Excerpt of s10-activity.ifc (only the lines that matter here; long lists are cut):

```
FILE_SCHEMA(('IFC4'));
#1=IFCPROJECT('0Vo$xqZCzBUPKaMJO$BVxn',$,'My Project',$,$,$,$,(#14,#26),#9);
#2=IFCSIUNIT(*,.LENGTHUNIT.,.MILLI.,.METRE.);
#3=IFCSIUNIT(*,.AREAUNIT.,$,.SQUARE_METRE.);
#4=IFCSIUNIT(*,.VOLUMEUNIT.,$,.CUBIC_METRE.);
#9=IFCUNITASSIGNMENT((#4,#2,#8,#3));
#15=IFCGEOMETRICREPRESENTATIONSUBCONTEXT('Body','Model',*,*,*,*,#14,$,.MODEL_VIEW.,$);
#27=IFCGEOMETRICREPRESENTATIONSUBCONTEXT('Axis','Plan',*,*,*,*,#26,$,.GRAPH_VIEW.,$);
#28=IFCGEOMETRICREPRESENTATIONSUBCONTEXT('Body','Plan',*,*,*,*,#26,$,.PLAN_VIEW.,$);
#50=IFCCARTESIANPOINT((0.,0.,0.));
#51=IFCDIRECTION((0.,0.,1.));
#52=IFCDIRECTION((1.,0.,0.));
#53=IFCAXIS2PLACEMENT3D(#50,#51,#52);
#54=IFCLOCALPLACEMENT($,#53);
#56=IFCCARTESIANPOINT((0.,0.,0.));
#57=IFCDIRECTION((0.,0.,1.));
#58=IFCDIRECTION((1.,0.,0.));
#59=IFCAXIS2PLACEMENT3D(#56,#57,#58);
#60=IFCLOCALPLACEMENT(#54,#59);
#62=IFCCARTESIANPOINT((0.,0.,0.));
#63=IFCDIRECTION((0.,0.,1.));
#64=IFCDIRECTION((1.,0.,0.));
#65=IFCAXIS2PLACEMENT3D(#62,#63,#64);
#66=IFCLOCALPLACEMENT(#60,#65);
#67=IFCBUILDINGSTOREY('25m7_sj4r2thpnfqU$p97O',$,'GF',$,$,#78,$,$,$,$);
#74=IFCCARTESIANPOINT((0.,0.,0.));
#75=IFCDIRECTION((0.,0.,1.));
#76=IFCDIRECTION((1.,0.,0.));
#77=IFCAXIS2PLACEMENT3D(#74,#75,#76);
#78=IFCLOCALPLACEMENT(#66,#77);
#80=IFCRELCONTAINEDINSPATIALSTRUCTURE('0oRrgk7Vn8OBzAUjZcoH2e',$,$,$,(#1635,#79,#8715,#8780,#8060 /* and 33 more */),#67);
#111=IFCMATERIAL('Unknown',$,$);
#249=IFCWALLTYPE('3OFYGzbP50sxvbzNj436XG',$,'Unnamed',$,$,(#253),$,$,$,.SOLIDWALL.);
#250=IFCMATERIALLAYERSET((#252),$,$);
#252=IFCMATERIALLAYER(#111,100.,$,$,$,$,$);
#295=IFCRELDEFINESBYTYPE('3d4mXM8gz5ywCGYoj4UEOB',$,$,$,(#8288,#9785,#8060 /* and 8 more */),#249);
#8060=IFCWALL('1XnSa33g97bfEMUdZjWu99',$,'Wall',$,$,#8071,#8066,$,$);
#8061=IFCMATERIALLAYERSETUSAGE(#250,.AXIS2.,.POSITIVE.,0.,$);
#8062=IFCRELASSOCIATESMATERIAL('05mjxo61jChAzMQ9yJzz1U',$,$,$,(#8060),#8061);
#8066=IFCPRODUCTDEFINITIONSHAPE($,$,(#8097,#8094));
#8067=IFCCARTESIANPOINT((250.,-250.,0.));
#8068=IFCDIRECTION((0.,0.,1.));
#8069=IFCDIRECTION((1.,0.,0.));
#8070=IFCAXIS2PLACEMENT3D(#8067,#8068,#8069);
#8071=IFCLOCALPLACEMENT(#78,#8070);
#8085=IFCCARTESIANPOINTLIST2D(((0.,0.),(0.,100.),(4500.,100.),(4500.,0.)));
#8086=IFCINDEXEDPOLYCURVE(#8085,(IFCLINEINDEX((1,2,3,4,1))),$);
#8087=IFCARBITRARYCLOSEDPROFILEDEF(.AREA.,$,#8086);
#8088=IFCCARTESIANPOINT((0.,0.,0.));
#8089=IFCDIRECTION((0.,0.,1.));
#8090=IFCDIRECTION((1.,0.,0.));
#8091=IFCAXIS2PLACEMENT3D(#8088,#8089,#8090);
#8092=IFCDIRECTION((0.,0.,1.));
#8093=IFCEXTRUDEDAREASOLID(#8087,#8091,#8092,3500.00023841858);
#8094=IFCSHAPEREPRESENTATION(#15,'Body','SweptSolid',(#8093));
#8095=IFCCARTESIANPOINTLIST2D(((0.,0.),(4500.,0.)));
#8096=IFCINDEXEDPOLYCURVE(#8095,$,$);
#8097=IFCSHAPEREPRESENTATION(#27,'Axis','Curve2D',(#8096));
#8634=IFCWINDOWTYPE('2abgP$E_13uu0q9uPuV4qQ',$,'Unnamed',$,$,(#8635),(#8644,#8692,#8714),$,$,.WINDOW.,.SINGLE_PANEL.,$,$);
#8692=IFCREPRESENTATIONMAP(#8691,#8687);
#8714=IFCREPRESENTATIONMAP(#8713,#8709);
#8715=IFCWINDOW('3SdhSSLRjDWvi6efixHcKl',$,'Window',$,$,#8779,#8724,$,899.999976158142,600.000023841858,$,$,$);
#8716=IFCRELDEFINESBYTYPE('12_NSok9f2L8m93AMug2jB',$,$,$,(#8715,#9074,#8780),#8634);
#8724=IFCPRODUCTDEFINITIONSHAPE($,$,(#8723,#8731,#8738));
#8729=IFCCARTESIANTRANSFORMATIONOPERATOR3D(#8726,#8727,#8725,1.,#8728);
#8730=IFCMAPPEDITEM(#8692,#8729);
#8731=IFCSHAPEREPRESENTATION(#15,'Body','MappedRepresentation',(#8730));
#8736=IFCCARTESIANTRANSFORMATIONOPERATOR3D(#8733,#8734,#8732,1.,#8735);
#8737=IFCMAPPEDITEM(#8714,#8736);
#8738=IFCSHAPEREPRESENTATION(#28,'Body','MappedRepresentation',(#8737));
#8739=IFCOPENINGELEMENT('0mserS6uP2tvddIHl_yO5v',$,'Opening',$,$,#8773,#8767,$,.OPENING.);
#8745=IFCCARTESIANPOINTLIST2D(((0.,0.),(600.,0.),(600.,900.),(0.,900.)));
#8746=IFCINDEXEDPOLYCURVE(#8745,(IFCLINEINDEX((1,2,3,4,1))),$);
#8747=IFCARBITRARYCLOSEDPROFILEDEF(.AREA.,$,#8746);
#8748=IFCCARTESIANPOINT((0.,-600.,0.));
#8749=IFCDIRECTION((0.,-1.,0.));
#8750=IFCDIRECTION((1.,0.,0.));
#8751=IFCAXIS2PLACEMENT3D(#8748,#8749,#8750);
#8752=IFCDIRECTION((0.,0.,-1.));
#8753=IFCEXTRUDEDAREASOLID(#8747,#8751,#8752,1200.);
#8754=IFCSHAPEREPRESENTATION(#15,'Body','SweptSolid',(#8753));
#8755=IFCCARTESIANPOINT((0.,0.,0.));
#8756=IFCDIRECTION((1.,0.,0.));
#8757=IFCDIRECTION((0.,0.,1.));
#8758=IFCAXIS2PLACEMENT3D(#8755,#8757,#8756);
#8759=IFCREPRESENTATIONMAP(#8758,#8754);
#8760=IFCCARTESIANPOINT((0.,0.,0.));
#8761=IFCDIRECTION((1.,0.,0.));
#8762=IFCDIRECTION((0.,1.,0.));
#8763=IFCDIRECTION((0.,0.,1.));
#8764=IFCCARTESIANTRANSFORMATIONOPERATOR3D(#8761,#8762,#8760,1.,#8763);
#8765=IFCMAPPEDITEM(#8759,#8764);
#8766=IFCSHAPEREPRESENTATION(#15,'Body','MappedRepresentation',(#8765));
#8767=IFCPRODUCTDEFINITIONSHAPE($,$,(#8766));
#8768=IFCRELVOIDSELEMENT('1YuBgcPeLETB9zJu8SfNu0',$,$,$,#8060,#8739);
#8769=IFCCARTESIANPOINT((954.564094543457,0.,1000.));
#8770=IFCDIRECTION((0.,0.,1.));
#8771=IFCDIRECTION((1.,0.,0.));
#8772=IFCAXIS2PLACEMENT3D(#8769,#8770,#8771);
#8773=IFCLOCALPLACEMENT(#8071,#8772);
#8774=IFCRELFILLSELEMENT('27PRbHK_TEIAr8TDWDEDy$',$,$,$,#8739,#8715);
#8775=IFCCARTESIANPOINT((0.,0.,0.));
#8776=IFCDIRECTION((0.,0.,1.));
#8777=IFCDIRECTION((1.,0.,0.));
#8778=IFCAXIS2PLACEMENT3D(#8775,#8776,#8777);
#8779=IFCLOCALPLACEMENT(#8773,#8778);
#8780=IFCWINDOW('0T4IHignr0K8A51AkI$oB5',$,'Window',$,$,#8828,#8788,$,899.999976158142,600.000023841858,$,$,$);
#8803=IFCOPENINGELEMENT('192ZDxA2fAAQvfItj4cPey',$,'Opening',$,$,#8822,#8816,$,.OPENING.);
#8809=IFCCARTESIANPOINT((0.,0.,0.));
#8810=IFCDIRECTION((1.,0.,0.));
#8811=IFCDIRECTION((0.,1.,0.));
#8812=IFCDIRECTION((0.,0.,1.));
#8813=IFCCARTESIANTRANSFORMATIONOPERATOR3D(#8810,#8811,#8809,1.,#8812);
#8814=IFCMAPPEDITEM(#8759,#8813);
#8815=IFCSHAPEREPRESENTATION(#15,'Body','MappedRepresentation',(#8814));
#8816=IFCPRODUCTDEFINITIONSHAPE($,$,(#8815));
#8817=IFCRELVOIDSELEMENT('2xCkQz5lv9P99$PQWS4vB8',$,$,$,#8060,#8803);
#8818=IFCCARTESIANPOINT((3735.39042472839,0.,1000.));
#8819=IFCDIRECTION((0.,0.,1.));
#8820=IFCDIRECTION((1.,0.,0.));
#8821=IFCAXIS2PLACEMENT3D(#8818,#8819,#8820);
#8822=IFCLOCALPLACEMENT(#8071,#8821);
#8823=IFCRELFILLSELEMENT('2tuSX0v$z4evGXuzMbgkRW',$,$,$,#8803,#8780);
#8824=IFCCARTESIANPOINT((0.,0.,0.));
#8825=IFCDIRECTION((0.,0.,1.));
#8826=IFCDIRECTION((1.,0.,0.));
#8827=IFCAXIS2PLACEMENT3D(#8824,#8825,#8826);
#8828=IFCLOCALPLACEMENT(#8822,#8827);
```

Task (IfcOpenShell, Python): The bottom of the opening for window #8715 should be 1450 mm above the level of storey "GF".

```python
import numpy as np
import ifcopenshell
import ifcopenshell.api.geometry
import ifcopenshell.geom
import ifcopenshell.util.element
import ifcopenshell.util.placement
import ifcopenshell.util.shape
import ifcopenshell.util.unit

model = ifcopenshell.open("s10-activity.ifc")
unit_scale = ifcopenshell.util.unit.calculate_unit_scale(model)

window = model.by_id(8715)
opening = window.FillsVoids[0].RelatingOpeningElement
storey = ifcopenshell.util.element.get_container(window, ifc_class="IfcBuildingStorey")
level = ifcopenshell.util.placement.get_local_placement(storey.ObjectPlacement)[2, 3]

# The opening's origin need not be at the sill, so measure its lowest point.
shape = ifcopenshell.geom.create_shape(ifcopenshell.geom.settings(), opening)
bottom = ifcopenshell.util.shape.get_shape_bottom_elevation(shape, shape.geometry) / unit_scale
dz = level + 1.45 / unit_scale - bottom

shift = np.array([0.0, 0.0, dz])
# The window is placed relative to its opening, so it follows when the opening moves.
matrix = ifcopenshell.util.placement.get_local_placement(opening.ObjectPlacement)
matrix[:3, 3] += shift
ifcopenshell.api.geometry.edit_object_placement(
    model, product=opening, matrix=matrix, is_si=False, should_transform_children=True
)

print(f"moved by {dz * unit_scale:+.3f} m")

model.write("s10-activity_edited.ifc")
```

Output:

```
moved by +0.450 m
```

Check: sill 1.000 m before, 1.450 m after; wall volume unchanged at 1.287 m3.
